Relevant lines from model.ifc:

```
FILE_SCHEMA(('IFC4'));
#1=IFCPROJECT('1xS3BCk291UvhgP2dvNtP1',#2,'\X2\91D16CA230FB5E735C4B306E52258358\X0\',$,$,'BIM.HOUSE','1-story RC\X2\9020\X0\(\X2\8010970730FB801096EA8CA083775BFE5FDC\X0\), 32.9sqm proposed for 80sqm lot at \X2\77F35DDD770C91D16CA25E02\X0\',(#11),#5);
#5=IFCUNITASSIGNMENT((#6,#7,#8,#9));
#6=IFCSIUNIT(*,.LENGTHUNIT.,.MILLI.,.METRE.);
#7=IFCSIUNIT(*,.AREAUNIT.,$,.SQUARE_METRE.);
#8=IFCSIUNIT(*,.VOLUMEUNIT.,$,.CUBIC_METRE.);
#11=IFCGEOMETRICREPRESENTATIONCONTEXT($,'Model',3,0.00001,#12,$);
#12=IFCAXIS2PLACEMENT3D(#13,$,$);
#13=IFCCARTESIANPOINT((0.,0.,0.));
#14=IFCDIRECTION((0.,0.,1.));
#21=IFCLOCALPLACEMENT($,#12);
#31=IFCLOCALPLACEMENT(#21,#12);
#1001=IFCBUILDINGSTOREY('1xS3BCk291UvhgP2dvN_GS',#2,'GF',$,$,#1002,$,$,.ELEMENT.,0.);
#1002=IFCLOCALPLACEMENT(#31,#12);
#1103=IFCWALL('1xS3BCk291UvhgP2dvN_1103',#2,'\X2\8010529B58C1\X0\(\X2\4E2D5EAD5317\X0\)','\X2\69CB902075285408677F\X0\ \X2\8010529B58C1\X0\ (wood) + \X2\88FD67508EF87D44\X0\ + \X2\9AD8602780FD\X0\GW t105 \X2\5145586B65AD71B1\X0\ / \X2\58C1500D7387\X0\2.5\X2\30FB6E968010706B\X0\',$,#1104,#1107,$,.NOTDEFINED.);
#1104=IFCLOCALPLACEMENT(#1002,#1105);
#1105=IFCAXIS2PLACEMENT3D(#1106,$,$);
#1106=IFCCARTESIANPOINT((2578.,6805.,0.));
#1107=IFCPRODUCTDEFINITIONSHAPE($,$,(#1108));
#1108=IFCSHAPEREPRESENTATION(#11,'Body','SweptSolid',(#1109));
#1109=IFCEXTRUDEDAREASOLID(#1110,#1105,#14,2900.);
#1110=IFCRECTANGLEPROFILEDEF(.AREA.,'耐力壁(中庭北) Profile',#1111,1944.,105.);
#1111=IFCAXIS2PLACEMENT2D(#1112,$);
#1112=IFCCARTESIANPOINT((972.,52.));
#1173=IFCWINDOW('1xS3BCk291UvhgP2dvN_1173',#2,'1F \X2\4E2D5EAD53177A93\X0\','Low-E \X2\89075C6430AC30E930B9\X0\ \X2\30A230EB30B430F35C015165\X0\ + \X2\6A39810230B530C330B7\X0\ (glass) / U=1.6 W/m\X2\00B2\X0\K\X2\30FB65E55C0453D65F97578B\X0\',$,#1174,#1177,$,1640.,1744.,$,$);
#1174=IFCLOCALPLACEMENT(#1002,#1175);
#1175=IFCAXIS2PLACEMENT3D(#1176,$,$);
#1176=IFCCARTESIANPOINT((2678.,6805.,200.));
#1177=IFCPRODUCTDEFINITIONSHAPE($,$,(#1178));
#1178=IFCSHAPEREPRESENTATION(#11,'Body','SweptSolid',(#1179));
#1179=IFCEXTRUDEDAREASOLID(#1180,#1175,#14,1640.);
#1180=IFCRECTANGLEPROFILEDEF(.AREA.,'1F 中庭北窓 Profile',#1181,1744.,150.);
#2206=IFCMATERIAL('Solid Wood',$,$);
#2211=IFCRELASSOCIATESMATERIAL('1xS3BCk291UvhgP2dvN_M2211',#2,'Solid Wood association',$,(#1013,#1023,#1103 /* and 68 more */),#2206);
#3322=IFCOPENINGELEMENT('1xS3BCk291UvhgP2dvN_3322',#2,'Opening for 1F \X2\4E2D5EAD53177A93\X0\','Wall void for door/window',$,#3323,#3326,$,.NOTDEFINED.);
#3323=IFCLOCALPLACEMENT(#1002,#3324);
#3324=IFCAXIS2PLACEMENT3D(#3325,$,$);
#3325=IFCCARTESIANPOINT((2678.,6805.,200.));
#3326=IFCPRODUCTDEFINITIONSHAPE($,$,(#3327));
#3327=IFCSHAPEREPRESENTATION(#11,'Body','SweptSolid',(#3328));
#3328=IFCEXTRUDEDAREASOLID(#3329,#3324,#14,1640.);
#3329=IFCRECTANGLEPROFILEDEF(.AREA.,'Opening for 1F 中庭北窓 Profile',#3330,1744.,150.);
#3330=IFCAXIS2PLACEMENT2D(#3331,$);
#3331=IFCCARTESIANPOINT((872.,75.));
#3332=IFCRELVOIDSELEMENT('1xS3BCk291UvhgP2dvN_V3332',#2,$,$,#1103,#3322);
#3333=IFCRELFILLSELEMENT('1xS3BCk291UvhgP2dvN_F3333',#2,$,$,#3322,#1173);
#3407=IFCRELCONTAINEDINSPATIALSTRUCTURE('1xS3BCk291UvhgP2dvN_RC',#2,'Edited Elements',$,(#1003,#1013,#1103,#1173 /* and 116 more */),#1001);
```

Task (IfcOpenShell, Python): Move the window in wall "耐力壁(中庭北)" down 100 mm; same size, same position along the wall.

```python
import numpy as np
import ifcopenshell
import ifcopenshell.api.geometry
import ifcopenshell.util.placement
import ifcopenshell.util.unit

model = ifcopenshell.open("model.ifc")
unit_scale = ifcopenshell.util.unit.calculate_unit_scale(model)

window = model.by_guid("1xS3BCk291UvhgP2dvN_1173")
opening = window.FillsVoids[0].RelatingOpeningElement
dz = -0.1 / unit_scale

shift = np.array([0.0, 0.0, dz])
# The window is not placed relative to its opening, so move both.
for product in (opening, window):
    matrix = ifcopenshell.util.placement.get_local_placement(product.ObjectPlacement)
    matrix[:3, 3] += shift
    ifcopenshell.api.geometry.edit_object_placement(model, product=product, matrix=matrix, is_si=False)

print(f"moved by {dz * unit_scale:+.3f} m")

model.write("model_v2.ifc")
```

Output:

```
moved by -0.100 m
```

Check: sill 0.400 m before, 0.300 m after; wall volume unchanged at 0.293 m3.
